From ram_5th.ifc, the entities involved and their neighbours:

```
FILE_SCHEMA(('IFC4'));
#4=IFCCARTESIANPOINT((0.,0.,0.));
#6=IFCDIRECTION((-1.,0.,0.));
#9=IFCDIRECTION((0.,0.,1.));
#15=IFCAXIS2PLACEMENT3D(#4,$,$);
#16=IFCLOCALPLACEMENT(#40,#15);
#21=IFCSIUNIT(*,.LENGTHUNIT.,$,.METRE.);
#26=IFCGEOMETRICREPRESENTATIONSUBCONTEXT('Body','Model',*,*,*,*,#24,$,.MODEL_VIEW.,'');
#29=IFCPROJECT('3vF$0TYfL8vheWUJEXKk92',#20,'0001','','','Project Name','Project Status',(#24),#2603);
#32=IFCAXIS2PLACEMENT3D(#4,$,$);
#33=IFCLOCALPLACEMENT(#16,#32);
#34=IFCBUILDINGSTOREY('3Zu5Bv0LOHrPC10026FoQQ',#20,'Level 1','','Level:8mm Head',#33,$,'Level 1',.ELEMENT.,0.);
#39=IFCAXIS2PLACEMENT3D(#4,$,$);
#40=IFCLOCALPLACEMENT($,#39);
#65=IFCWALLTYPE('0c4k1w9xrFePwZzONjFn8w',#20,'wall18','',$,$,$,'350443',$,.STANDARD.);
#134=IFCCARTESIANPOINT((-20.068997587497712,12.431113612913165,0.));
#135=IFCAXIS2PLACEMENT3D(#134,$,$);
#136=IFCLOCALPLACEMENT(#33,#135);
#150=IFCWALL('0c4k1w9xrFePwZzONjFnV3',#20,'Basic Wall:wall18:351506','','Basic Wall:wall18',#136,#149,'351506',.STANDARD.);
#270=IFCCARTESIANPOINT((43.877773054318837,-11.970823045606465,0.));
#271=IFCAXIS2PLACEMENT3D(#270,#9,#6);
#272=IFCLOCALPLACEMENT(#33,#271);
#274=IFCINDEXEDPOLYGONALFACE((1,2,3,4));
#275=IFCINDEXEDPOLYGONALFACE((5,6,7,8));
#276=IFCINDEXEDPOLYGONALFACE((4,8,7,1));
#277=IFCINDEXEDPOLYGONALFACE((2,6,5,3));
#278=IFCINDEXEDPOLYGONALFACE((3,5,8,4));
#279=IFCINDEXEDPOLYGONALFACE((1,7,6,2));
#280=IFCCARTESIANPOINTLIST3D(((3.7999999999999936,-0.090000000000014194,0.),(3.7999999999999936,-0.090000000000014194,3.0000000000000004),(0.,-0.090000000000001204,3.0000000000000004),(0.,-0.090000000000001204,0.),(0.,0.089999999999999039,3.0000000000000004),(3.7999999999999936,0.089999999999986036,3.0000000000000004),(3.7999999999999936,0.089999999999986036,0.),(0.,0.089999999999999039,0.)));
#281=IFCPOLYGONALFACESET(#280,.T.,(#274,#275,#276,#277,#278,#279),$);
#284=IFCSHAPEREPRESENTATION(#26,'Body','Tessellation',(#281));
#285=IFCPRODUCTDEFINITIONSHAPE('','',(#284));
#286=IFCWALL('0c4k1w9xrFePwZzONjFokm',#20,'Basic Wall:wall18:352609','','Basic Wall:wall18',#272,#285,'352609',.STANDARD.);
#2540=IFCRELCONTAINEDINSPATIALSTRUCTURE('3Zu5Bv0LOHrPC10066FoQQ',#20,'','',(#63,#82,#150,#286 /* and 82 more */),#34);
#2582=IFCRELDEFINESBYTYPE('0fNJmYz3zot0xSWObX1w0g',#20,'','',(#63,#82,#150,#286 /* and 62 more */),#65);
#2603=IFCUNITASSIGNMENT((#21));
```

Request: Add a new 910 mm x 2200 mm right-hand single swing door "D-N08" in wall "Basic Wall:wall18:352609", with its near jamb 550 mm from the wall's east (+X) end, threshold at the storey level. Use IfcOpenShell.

```python
import numpy as np
import ifcopenshell
import ifcopenshell.api.feature
import ifcopenshell.api.geometry
import ifcopenshell.api.root
import ifcopenshell.api.spatial
import ifcopenshell.geom
import ifcopenshell.util.element
import ifcopenshell.util.placement
import ifcopenshell.util.representation
import ifcopenshell.util.shape
import ifcopenshell.util.unit

model = ifcopenshell.open("ram_5th.ifc")
unit_scale = ifcopenshell.util.unit.calculate_unit_scale(model)
settings = ifcopenshell.geom.settings()


def volume(element):
    """Net volume in cubic metres, openings subtracted."""
    shape = ifcopenshell.geom.create_shape(settings, element)
    return ifcopenshell.util.shape.get_volume(shape.geometry)


wall = model.by_guid("0c4k1w9xrFePwZzONjFokm")
storey = ifcopenshell.util.element.get_container(wall, ifc_class="IfcBuildingStorey")
context = ifcopenshell.util.representation.get_context(model, "Model", "Body", "MODEL_VIEW")
before = volume(wall)

width, height, from_end, sill = 0.91, 2.2, 0.55, 0.0  # metres

# The wall runs along its own X axis, and the end named is its -X end.
wall_shape = ifcopenshell.geom.create_shape(settings, wall)
x, y, z = ifcopenshell.util.shape.get_vertices(wall_shape.geometry).T
start = x.min() + from_end
face, thickness = float(y.min()), float(y.max() - y.min())
wall_matrix = ifcopenshell.util.placement.get_local_placement(wall.ObjectPlacement)
level = ifcopenshell.util.placement.get_local_placement(storey.ObjectPlacement)[2, 3]


def in_wall(x, y):
    """Placement at x, y metres in the wall's axes, at sill height."""
    matrix = wall_matrix.copy()
    matrix[:, 3] = wall_matrix @ np.array([x / unit_scale, y / unit_scale, 0.0, 1.0])
    matrix[2, 3] = level + sill / unit_scale
    return matrix


# Opening: a box that overshoots both wall faces by 50 mm.
opening = ifcopenshell.api.root.create_entity(model, ifc_class="IfcOpeningElement", predefined_type="OPENING")
box = ifcopenshell.api.geometry.add_wall_representation(
    model, context=context, length=width, height=height, thickness=thickness + 0.1
)
ifcopenshell.api.geometry.assign_representation(model, product=opening, representation=box)
ifcopenshell.api.geometry.edit_object_placement(model, product=opening, matrix=in_wall(start, face - 0.05), is_si=False)
ifcopenshell.api.feature.add_feature(model, feature=opening, element=wall)

door = ifcopenshell.api.root.create_entity(model, ifc_class="IfcDoor", name="D-N08", predefined_type="DOOR")
door.OverallWidth, door.OverallHeight = width / unit_scale, height / unit_scale
door.OperationType = "SINGLE_SWING_RIGHT"
body = ifcopenshell.api.geometry.add_door_representation(
    model,
    context=context,
    overall_width=door.OverallWidth,
    overall_height=door.OverallHeight,
    operation_type="SINGLE_SWING_RIGHT",
    lining_properties={"LiningDepth": thickness / unit_scale, "ThresholdDepth": thickness / unit_scale},
)
ifcopenshell.api.geometry.assign_representation(model, product=door, representation=body)
ifcopenshell.api.spatial.assign_container(model, products=[door], relating_structure=storey)
ifcopenshell.api.feature.add_filling(model, opening=opening, element=door)

# The lining spans the wall, so the door starts at the wall face.
ifcopenshell.api.geometry.edit_object_placement(model, product=door, matrix=in_wall(start, face), is_si=False)

after = volume(wall)

print(f"wall volume {before:.3f} -> {after:.3f} m3")

model.write("ram_5th_updated.ifc")
```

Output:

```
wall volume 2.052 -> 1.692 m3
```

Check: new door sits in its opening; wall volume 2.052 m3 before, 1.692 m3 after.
